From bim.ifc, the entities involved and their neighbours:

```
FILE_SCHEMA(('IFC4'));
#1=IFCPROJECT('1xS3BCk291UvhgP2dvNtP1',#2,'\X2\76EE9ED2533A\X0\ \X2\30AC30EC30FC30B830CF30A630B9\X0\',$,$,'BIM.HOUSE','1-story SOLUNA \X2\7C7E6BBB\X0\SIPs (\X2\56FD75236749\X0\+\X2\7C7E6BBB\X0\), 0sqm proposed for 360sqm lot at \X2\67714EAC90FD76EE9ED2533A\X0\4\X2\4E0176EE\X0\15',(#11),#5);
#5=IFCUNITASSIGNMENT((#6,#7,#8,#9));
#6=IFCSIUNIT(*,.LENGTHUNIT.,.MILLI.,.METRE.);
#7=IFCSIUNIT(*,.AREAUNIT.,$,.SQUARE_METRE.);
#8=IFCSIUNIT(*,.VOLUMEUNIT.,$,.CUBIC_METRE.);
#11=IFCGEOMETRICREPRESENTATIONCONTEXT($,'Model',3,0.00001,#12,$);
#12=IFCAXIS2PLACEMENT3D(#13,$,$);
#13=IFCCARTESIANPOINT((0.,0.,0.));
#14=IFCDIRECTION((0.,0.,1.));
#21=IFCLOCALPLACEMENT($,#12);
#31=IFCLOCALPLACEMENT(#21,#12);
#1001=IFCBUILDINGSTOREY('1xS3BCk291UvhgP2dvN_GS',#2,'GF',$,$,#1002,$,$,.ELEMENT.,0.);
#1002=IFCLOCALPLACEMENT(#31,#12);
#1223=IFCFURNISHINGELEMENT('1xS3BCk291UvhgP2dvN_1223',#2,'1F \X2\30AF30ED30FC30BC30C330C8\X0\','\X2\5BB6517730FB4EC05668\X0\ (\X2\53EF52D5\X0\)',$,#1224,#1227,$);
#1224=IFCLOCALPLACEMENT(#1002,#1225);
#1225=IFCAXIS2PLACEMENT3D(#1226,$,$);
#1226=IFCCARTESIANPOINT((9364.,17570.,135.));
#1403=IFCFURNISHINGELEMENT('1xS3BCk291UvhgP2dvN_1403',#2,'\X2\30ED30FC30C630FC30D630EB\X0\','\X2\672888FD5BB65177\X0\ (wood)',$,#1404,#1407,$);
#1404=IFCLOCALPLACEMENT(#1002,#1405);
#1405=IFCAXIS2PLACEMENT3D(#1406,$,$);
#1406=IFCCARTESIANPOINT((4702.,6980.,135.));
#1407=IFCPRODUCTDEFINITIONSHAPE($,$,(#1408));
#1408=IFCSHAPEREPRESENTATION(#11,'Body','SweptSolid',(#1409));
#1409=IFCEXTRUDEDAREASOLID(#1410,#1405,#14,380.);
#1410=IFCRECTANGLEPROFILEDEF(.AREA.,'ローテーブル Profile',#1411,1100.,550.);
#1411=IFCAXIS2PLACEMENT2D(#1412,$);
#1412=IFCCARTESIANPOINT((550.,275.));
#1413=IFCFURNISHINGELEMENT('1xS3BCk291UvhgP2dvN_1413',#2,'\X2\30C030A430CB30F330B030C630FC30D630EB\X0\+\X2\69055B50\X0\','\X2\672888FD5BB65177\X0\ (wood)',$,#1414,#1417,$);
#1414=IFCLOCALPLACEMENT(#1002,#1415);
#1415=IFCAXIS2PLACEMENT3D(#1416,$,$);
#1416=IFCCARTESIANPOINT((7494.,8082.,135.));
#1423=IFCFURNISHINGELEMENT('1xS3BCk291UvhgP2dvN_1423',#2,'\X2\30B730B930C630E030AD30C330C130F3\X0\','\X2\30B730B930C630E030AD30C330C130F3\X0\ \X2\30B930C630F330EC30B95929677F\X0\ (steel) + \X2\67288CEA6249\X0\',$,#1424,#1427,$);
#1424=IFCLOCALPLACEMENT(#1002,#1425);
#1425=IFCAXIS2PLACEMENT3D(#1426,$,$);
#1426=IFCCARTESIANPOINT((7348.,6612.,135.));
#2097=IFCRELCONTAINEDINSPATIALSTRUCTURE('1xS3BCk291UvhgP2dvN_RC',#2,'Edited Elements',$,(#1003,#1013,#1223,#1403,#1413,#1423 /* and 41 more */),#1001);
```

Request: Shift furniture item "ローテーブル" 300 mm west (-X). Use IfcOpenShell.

```python
import ifcopenshell
import ifcopenshell.api.geometry
import ifcopenshell.util.placement
import ifcopenshell.util.unit

model = ifcopenshell.open("bim.ifc")
unit_scale = ifcopenshell.util.unit.calculate_unit_scale(model)

item = model.by_guid("1xS3BCk291UvhgP2dvN_1403")
matrix = ifcopenshell.util.placement.get_local_placement(item.ObjectPlacement)
matrix[0, 3] -= 0.3 / unit_scale
ifcopenshell.api.geometry.edit_object_placement(model, product=item, matrix=matrix, is_si=False)

print(ifcopenshell.util.placement.get_local_placement(item.ObjectPlacement).round(3) + 0.0)

model.write("bim_updated.ifc")
```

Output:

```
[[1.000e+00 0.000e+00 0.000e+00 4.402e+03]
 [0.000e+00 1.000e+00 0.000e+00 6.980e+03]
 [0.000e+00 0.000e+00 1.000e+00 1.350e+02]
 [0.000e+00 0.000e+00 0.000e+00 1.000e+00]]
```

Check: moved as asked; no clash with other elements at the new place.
